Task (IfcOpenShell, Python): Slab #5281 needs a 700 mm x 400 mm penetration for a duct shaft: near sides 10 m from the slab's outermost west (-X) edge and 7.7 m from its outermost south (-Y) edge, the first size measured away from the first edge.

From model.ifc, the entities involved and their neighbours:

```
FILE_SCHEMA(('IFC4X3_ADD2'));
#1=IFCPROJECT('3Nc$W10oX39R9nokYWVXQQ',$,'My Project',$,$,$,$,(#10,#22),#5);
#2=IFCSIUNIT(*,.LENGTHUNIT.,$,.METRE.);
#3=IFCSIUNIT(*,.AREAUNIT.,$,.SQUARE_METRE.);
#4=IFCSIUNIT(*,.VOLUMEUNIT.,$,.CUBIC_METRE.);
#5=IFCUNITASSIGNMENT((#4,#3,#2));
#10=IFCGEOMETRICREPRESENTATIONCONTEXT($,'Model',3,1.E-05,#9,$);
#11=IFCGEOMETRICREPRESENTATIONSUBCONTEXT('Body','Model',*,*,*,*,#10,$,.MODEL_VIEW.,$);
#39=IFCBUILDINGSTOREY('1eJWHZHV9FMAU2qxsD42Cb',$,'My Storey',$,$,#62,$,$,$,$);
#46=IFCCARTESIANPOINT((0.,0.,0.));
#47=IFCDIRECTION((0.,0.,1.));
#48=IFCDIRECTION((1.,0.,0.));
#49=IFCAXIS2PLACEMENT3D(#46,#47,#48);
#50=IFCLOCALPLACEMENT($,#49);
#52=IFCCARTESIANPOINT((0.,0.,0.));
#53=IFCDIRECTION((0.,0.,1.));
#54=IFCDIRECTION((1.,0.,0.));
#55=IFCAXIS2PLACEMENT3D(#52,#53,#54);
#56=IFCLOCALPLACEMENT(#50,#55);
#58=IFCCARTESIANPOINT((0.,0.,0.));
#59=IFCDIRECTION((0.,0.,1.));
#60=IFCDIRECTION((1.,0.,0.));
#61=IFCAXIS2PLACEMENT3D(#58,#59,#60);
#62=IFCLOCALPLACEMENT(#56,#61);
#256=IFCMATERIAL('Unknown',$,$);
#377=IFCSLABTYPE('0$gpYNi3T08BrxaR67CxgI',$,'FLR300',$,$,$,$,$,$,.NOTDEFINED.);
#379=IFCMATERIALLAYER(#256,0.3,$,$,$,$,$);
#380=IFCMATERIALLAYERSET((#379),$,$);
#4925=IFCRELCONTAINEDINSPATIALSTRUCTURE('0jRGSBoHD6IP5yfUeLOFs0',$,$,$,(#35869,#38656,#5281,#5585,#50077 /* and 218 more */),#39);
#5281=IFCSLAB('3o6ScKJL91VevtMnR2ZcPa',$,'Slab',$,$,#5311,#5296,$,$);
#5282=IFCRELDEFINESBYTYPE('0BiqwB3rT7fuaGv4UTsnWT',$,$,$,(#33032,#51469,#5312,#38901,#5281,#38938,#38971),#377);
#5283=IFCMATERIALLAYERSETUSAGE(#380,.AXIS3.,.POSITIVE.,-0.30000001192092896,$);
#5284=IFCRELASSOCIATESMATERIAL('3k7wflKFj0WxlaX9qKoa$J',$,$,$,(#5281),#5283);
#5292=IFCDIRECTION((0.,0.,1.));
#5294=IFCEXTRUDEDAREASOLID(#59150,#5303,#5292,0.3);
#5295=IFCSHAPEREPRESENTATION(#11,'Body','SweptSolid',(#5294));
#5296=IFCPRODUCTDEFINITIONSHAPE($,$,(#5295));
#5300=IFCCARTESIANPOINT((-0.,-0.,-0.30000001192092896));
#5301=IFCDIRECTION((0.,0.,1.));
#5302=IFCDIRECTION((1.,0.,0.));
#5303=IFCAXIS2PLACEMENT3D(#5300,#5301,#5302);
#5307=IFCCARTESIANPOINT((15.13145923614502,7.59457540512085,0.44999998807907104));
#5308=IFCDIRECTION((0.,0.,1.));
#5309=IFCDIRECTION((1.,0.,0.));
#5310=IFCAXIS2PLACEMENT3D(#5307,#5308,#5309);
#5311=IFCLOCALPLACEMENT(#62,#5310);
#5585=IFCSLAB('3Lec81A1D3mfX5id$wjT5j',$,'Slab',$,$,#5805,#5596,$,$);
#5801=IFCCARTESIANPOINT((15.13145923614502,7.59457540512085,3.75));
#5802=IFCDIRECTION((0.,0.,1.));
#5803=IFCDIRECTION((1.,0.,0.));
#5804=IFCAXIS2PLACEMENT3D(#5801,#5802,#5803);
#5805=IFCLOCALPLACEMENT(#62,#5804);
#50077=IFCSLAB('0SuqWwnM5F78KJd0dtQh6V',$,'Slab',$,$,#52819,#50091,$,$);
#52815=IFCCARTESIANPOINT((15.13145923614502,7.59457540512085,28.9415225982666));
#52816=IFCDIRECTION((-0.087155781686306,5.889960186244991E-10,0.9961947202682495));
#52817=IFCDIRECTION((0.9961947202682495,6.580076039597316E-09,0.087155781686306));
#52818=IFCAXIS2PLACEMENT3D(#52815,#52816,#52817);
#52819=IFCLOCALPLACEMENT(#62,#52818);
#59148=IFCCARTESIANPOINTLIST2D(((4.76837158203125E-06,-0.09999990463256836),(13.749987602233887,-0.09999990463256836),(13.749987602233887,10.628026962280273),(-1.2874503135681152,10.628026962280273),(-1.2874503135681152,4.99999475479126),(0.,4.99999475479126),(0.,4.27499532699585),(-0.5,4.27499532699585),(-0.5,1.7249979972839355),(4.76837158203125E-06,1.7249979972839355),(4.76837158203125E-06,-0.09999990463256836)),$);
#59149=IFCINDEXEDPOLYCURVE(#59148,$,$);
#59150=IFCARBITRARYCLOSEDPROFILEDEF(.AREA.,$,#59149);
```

```python
import numpy as np
import ifcopenshell
import ifcopenshell.api.feature
import ifcopenshell.api.geometry
import ifcopenshell.api.root
import ifcopenshell.geom
import ifcopenshell.util.placement
import ifcopenshell.util.representation
import ifcopenshell.util.shape
import ifcopenshell.util.unit

model = ifcopenshell.open("model.ifc")
unit_scale = ifcopenshell.util.unit.calculate_unit_scale(model)
settings = ifcopenshell.geom.settings()


def volume(element):
    """Net volume in cubic metres, openings subtracted."""
    shape = ifcopenshell.geom.create_shape(settings, element)
    return ifcopenshell.util.shape.get_volume(shape.geometry)


slab = model.by_guid("3o6ScKJL91VevtMnR2ZcPa")
before = volume(slab)

# Extent in the slab's own axes, in metres. The edges named are its -X and -Y sides.
slab_shape = ifcopenshell.geom.create_shape(settings, slab)
vertices = ifcopenshell.util.shape.get_vertices(slab_shape.geometry)
x_min, y_min, bottom = vertices.min(axis=0)
top = vertices[:, 2].max()

opening = ifcopenshell.api.root.create_entity(model, ifc_class="IfcOpeningElement", name="Duct shaft opening", predefined_type="OPENING")
context = ifcopenshell.util.representation.get_context(model, "Model", "Body", "MODEL_VIEW")
width, depth = 0.7, 0.4
outline = [(0.0, 0.0), (width, 0.0), (width, depth), (0.0, depth), (0.0, 0.0)]
# Overshoot both faces by 50 mm so the cut is clean.
shape = ifcopenshell.api.geometry.add_slab_representation(
    model, context=context, depth=top - bottom + 0.1, polyline=outline
)
ifcopenshell.api.geometry.assign_representation(model, product=opening, representation=shape)

matrix = ifcopenshell.util.placement.get_local_placement(slab.ObjectPlacement)
matrix[:, 3] = matrix @ np.append(np.array([x_min + 10, y_min + 7.7, bottom - 0.05]) / unit_scale, 1.0)
ifcopenshell.api.geometry.edit_object_placement(model, product=opening, matrix=matrix, is_si=False)
ifcopenshell.api.feature.add_feature(model, feature=opening, element=slab)

after = volume(slab)

print(f"slab volume {before:.3f} -> {after:.3f} m3")

model.write("model_edited.ifc")
```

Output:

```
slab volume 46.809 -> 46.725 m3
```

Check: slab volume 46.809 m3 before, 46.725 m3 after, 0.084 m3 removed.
